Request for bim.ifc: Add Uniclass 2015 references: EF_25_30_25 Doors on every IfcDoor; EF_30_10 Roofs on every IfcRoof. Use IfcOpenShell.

First a look at what the model holds.

```python
import ifcopenshell

model = ifcopenshell.open("bim.ifc")
print(model.schema)
print("classifications:", [c.Name for c in model.by_type("IfcClassification")])
for ifc_class in ("IfcDoor", "IfcRoof", "IfcStair", "IfcWall", "IfcWindow"):
    print(ifc_class, len(model.by_type(ifc_class)))
```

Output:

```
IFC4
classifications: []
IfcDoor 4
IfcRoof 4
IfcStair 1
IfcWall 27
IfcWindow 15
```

```python
import ifcopenshell
import ifcopenshell.api.classification

model = ifcopenshell.open("bim.ifc")

system = ifcopenshell.api.classification.add_classification(model, classification="Uniclass 2015")

codes = {
    "IfcDoor": ("EF_25_30_25", "Doors"),
    "IfcRoof": ("EF_30_10", "Roofs"),
}
for ifc_class, (code, name) in codes.items():
    products = model.by_type(ifc_class)
    ifcopenshell.api.classification.add_reference(
        model, products=products, classification=system, identification=code, name=name
    )
    print(code, len(products))

model.write("bim_v2.ifc")
```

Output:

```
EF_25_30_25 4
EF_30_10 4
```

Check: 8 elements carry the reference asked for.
